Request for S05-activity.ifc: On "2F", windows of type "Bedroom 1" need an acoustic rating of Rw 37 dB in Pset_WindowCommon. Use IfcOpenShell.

First a look at what the model holds.

```python
import ifcopenshell
import ifcopenshell.util.element

model = ifcopenshell.open("S05-activity.ifc")
print(model.schema)
storey = next(s for s in model.by_type("IfcBuildingStorey") if s.Name == "2F")
windows = [e for e in ifcopenshell.util.element.get_decomposition(storey) if e.is_a("IfcWindow")]
seen = {}
for e in windows:
    element_type = ifcopenshell.util.element.get_type(e)
    key = (element_type.Name if element_type != e and element_type else None, ifcopenshell.util.element.get_pset(e, "Pset_WindowCommon", "AcousticRating"))
    seen[key] = seen.get(key, 0) + 1
for (name, value), count in sorted(seen.items(), key=str):
    print(count, "x", name, "|", value)
```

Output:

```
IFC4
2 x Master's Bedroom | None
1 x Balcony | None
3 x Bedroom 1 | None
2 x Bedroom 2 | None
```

```python
import ifcopenshell
import ifcopenshell.api.pset
import ifcopenshell.util.element

model = ifcopenshell.open("S05-activity.ifc")

storey = next(s for s in model.by_type("IfcBuildingStorey") if s.Name == "2F")
windows = [e for e in ifcopenshell.util.element.get_decomposition(storey) if e.is_a("IfcWindow")]

count = 0
for e in windows:
    element_type = ifcopenshell.util.element.get_type(e)
    if element_type in (None, e) or element_type.Name != "Bedroom 1":
        continue
    # add_pset returns the element's existing set when there is one.
    pset = ifcopenshell.api.pset.add_pset(model, product=e, name="Pset_WindowCommon")
    ifcopenshell.api.pset.edit_pset(model, pset=pset, properties={"AcousticRating": "Rw 37 dB"})
    count += 1

print(count, "windows updated")

model.write("S05-activity-out.ifc")
```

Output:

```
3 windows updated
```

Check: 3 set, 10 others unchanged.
